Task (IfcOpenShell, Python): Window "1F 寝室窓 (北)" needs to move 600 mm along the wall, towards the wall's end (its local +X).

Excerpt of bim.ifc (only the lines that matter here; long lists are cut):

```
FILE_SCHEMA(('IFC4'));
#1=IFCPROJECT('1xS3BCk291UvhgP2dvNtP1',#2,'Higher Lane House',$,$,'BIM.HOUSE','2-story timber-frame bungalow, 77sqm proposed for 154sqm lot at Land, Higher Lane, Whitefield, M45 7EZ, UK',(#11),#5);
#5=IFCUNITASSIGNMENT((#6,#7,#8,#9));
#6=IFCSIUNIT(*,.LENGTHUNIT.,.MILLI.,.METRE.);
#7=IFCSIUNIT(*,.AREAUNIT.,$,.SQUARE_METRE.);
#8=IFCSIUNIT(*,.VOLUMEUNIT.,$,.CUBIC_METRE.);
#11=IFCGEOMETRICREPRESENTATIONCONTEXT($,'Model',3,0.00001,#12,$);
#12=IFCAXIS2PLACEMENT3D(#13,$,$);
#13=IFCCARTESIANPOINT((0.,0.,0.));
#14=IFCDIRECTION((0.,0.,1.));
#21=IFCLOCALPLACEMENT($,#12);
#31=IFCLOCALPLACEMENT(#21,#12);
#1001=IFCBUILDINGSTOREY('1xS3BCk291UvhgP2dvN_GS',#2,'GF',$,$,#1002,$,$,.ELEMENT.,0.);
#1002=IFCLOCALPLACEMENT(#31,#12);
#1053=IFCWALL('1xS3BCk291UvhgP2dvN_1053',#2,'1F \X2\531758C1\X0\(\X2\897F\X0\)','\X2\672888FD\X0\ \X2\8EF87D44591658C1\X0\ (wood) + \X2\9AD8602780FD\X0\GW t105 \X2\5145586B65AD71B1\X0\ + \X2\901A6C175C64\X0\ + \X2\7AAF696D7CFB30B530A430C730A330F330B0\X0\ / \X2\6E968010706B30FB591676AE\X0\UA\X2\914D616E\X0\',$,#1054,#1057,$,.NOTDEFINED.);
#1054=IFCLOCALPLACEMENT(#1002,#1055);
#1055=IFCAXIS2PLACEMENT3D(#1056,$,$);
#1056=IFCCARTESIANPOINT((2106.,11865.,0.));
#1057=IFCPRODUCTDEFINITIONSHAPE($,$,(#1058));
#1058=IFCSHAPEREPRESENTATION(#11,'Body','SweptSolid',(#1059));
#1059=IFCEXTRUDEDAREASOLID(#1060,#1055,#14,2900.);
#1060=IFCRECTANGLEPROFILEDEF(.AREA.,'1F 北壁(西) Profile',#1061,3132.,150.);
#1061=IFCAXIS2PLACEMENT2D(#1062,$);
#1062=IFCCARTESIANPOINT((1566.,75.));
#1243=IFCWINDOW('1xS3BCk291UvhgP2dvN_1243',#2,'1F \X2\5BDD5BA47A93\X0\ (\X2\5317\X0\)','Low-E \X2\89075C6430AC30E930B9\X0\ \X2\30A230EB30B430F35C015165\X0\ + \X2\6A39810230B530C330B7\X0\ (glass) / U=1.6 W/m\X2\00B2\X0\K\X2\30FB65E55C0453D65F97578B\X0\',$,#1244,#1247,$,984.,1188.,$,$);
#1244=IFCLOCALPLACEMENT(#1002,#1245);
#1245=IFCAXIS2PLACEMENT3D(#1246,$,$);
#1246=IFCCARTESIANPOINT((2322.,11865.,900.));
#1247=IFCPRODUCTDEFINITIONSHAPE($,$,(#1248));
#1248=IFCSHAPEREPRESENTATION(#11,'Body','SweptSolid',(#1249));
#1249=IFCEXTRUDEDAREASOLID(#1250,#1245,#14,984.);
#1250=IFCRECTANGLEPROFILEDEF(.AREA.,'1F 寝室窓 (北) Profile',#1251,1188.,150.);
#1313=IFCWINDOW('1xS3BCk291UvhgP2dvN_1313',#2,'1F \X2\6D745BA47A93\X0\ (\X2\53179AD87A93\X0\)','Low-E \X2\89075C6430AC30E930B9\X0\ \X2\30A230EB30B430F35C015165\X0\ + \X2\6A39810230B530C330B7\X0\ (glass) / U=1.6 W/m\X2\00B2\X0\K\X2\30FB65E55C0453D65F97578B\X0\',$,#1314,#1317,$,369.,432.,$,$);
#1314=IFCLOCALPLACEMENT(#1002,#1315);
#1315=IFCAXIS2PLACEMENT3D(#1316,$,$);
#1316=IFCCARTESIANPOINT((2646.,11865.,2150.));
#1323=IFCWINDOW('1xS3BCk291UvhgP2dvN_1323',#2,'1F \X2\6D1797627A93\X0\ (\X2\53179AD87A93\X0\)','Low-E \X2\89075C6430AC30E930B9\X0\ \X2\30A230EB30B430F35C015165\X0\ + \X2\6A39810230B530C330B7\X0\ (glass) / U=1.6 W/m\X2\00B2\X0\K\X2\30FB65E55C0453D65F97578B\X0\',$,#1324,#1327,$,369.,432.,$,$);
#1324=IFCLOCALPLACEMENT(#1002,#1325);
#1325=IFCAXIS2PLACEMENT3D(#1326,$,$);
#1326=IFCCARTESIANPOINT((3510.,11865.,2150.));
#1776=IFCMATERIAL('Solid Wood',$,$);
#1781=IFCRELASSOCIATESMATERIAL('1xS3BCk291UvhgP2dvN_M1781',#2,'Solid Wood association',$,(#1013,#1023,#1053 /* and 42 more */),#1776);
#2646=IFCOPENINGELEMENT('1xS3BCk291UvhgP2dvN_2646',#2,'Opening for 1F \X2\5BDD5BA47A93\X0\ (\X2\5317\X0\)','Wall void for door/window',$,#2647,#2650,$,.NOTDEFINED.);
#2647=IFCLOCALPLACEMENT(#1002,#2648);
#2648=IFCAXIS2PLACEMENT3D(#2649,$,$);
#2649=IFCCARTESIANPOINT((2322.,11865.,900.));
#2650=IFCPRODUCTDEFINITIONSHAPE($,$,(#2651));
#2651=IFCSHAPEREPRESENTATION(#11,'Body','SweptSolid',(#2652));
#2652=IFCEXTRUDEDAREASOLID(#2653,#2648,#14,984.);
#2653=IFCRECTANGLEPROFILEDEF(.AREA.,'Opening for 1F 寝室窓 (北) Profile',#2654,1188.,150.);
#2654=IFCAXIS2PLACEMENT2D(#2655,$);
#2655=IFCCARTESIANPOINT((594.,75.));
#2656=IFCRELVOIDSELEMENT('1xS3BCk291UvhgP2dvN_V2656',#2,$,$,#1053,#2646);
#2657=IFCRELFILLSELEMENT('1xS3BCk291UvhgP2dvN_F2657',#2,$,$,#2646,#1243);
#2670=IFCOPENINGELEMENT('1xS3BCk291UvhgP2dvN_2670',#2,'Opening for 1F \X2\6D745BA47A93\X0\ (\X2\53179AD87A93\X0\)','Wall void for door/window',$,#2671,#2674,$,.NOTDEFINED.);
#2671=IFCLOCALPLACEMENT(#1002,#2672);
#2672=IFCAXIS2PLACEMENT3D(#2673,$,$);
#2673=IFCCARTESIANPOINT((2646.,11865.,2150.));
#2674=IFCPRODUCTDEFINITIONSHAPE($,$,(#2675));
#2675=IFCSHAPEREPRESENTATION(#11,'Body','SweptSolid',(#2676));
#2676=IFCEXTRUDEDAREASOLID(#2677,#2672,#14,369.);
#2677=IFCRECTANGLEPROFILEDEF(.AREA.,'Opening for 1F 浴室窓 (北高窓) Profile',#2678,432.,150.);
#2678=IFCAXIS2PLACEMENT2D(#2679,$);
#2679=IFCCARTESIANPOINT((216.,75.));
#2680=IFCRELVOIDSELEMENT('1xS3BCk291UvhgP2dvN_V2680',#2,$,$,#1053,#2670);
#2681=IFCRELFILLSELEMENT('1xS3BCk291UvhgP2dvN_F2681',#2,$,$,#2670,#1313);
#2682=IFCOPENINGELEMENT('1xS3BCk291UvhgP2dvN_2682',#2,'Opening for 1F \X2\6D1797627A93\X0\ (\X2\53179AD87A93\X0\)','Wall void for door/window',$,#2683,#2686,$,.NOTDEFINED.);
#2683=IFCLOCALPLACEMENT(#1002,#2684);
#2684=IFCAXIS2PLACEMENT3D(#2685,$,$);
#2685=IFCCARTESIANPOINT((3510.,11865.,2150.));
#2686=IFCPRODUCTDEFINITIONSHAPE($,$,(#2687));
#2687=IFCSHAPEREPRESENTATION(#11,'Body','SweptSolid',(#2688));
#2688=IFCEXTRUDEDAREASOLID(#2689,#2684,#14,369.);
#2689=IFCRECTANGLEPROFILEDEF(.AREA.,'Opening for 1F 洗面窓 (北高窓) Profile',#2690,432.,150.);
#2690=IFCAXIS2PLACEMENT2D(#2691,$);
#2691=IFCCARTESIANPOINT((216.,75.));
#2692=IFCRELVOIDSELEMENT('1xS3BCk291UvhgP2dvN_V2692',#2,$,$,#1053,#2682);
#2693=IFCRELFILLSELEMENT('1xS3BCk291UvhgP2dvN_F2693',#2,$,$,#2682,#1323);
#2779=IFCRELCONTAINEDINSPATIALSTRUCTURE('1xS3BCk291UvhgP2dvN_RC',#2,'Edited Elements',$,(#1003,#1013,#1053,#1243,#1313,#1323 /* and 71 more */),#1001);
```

```python
import ifcopenshell
import ifcopenshell.api.geometry
import ifcopenshell.util.placement

model = ifcopenshell.open("bim.ifc")

window = model.by_guid("1xS3BCk291UvhgP2dvN_1243")
opening = window.FillsVoids[0].RelatingOpeningElement
wall = opening.VoidsElements[0].RelatingBuildingElement

wall_matrix = ifcopenshell.util.placement.get_local_placement(wall.ObjectPlacement)
shift = wall_matrix[:3, 0] * 600.0
before = ifcopenshell.util.placement.get_local_placement(window.ObjectPlacement)[:3, 3].copy()

# The window is not placed relative to its opening, so move both.
for product in (opening, window):
    matrix = ifcopenshell.util.placement.get_local_placement(product.ObjectPlacement)
    matrix[:3, 3] += shift
    ifcopenshell.api.geometry.edit_object_placement(model, product=product, matrix=matrix, is_si=False)

after = ifcopenshell.util.placement.get_local_placement(window.ObjectPlacement)[:3, 3]
print("window moved by", (after - before).round(3) + 0.0)

model.write("bim_updated.ifc")
```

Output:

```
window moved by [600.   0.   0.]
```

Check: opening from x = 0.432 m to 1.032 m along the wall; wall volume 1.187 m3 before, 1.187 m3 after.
